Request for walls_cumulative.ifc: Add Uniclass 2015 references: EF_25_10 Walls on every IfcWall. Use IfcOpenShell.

First a look at what the model holds.

```python
import ifcopenshell

model = ifcopenshell.open("walls_cumulative.ifc")
print(model.schema)
print("classifications:", [c.Name for c in model.by_type("IfcClassification")])
for ifc_class in ("IfcDoor", "IfcRoof", "IfcStair", "IfcWall", "IfcWindow"):
    print(ifc_class, len(model.by_type(ifc_class)))
```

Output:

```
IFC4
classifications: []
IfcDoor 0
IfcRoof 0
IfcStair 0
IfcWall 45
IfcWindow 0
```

```python
import ifcopenshell
import ifcopenshell.api.classification

model = ifcopenshell.open("walls_cumulative.ifc")

system = ifcopenshell.api.classification.add_classification(model, classification="Uniclass 2015")

codes = {
    "IfcWall": ("EF_25_10", "Walls"),
}
for ifc_class, (code, name) in codes.items():
    products = model.by_type(ifc_class)
    ifcopenshell.api.classification.add_reference(
        model, products=products, classification=system, identification=code, name=name
    )
    print(code, len(products))

model.write("walls_cumulative_updated.ifc")
```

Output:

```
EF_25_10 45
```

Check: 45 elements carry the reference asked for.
